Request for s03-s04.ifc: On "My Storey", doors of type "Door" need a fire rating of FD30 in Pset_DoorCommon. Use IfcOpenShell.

First a look at what the model holds.

```python
import ifcopenshell
import ifcopenshell.util.element

model = ifcopenshell.open("s03-s04.ifc")
print(model.schema)
storey = next(s for s in model.by_type("IfcBuildingStorey") if s.Name == "My Storey")
doors = [e for e in ifcopenshell.util.element.get_decomposition(storey) if e.is_a("IfcDoor")]
seen = {}
for e in doors:
    element_type = ifcopenshell.util.element.get_type(e)
    key = (element_type.Name if element_type != e and element_type else None, ifcopenshell.util.element.get_pset(e, "Pset_DoorCommon", "FireRating"))
    seen[key] = seen.get(key, 0) + 1
for (name, value), count in sorted(seen.items(), key=str):
    print(count, "x", name, "|", value)
```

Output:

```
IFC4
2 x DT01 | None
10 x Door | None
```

```python
import ifcopenshell
import ifcopenshell.api.pset
import ifcopenshell.util.element

model = ifcopenshell.open("s03-s04.ifc")

storey = next(s for s in model.by_type("IfcBuildingStorey") if s.Name == "My Storey")
doors = [e for e in ifcopenshell.util.element.get_decomposition(storey) if e.is_a("IfcDoor")]

count = 0
for e in doors:
    element_type = ifcopenshell.util.element.get_type(e)
    if element_type in (None, e) or element_type.Name != "Door":
        continue
    # add_pset returns the element's existing set when there is one.
    pset = ifcopenshell.api.pset.add_pset(model, product=e, name="Pset_DoorCommon")
    ifcopenshell.api.pset.edit_pset(model, pset=pset, properties={"FireRating": "FD30"})
    count += 1

print(count, "doors updated")

model.write("s03-s04_rev.ifc")
```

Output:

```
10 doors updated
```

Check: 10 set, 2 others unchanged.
